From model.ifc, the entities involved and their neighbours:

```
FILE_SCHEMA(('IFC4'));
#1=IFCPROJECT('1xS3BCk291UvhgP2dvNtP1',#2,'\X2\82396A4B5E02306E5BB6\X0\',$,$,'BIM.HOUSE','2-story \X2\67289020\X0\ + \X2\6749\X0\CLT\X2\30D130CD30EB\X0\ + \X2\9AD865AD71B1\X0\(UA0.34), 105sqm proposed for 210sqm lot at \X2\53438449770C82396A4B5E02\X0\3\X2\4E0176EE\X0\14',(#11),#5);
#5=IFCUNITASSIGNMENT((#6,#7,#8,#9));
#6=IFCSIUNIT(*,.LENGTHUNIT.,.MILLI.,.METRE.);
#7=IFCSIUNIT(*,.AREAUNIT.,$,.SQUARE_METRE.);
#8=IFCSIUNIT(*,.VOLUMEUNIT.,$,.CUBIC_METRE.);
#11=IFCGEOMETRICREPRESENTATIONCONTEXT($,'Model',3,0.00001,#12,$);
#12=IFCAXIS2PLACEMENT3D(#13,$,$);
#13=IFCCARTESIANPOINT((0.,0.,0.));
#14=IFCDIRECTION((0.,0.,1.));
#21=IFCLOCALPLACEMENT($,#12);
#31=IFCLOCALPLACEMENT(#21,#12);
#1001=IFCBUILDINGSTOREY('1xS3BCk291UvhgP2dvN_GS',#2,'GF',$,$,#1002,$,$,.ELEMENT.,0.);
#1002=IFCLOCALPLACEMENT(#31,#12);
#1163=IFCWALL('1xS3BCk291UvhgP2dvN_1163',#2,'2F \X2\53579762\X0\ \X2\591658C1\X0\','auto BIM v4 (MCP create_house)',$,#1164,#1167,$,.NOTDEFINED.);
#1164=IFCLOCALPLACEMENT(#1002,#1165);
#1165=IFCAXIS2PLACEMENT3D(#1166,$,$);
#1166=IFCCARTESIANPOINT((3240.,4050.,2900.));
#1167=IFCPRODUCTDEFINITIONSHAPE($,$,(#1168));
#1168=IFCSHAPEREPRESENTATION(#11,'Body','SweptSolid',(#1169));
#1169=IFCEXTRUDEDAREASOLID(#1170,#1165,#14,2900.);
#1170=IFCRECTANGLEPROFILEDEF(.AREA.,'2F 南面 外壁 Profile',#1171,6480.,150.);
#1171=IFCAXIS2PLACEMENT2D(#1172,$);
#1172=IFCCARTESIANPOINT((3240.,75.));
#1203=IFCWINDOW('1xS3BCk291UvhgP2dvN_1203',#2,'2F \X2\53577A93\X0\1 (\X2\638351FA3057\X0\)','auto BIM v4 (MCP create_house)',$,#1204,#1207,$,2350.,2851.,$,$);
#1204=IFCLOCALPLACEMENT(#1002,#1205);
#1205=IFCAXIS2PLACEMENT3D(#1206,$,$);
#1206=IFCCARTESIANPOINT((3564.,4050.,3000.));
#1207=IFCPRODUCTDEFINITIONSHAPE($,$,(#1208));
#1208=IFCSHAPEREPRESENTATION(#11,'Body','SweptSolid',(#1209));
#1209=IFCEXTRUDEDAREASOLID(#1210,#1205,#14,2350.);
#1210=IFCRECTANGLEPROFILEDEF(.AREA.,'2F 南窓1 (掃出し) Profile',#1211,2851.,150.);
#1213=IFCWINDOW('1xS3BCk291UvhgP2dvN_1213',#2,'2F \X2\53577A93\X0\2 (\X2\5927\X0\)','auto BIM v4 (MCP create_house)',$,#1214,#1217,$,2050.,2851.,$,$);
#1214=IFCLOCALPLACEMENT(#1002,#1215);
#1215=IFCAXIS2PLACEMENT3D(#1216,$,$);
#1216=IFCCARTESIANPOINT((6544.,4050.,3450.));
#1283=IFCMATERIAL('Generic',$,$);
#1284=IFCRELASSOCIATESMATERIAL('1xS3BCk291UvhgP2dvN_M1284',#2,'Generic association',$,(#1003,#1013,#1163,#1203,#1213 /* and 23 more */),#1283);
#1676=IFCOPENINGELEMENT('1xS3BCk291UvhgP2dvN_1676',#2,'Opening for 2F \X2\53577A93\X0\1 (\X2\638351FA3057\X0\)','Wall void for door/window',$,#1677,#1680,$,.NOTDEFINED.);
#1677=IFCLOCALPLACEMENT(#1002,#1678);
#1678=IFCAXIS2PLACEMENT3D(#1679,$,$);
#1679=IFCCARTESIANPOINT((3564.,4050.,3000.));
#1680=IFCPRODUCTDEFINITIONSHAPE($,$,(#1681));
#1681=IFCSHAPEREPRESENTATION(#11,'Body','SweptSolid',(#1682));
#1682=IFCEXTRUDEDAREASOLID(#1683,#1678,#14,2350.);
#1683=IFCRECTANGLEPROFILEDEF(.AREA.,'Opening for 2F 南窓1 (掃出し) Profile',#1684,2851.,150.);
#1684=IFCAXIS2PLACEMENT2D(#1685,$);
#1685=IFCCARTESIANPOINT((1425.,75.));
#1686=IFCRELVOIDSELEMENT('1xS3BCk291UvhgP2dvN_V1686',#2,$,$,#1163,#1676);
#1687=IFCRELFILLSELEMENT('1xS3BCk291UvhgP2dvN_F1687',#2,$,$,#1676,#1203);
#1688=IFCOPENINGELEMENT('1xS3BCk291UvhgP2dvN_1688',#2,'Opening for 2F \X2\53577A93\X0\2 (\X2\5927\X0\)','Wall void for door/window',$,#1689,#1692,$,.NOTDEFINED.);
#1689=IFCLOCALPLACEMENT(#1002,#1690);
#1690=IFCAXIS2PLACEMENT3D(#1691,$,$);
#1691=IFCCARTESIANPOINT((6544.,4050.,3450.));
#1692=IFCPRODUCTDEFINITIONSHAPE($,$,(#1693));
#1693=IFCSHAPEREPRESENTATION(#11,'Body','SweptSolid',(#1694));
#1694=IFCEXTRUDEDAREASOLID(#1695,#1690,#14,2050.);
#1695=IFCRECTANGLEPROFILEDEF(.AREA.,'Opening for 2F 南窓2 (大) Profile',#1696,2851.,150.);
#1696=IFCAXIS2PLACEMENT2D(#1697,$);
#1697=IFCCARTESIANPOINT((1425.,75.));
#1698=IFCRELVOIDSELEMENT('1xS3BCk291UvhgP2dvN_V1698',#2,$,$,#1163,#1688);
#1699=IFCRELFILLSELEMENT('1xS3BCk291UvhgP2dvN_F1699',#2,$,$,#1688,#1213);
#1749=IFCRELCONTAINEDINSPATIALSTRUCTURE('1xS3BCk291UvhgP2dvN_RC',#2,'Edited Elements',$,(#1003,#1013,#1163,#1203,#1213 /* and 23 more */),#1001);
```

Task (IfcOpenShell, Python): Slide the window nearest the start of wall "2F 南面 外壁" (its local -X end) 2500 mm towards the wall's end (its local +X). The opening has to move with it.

```python
import ifcopenshell
import ifcopenshell.api.geometry
import ifcopenshell.util.placement

model = ifcopenshell.open("model.ifc")

window = model.by_guid("1xS3BCk291UvhgP2dvN_1203")
opening = window.FillsVoids[0].RelatingOpeningElement
wall = opening.VoidsElements[0].RelatingBuildingElement

wall_matrix = ifcopenshell.util.placement.get_local_placement(wall.ObjectPlacement)
shift = wall_matrix[:3, 0] * 2500.0
before = ifcopenshell.util.placement.get_local_placement(window.ObjectPlacement)[:3, 3].copy()

# The window is not placed relative to its opening, so move both.
for product in (opening, window):
    matrix = ifcopenshell.util.placement.get_local_placement(product.ObjectPlacement)
    matrix[:3, 3] += shift
    ifcopenshell.api.geometry.edit_object_placement(model, product=product, matrix=matrix, is_si=False)

after = ifcopenshell.util.placement.get_local_placement(window.ObjectPlacement)[:3, 3]
print("window moved by", (after - before).round(3) + 0.0)

model.write("model_edited.ifc")
```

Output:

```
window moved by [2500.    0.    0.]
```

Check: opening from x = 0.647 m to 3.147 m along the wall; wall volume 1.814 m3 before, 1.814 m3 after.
